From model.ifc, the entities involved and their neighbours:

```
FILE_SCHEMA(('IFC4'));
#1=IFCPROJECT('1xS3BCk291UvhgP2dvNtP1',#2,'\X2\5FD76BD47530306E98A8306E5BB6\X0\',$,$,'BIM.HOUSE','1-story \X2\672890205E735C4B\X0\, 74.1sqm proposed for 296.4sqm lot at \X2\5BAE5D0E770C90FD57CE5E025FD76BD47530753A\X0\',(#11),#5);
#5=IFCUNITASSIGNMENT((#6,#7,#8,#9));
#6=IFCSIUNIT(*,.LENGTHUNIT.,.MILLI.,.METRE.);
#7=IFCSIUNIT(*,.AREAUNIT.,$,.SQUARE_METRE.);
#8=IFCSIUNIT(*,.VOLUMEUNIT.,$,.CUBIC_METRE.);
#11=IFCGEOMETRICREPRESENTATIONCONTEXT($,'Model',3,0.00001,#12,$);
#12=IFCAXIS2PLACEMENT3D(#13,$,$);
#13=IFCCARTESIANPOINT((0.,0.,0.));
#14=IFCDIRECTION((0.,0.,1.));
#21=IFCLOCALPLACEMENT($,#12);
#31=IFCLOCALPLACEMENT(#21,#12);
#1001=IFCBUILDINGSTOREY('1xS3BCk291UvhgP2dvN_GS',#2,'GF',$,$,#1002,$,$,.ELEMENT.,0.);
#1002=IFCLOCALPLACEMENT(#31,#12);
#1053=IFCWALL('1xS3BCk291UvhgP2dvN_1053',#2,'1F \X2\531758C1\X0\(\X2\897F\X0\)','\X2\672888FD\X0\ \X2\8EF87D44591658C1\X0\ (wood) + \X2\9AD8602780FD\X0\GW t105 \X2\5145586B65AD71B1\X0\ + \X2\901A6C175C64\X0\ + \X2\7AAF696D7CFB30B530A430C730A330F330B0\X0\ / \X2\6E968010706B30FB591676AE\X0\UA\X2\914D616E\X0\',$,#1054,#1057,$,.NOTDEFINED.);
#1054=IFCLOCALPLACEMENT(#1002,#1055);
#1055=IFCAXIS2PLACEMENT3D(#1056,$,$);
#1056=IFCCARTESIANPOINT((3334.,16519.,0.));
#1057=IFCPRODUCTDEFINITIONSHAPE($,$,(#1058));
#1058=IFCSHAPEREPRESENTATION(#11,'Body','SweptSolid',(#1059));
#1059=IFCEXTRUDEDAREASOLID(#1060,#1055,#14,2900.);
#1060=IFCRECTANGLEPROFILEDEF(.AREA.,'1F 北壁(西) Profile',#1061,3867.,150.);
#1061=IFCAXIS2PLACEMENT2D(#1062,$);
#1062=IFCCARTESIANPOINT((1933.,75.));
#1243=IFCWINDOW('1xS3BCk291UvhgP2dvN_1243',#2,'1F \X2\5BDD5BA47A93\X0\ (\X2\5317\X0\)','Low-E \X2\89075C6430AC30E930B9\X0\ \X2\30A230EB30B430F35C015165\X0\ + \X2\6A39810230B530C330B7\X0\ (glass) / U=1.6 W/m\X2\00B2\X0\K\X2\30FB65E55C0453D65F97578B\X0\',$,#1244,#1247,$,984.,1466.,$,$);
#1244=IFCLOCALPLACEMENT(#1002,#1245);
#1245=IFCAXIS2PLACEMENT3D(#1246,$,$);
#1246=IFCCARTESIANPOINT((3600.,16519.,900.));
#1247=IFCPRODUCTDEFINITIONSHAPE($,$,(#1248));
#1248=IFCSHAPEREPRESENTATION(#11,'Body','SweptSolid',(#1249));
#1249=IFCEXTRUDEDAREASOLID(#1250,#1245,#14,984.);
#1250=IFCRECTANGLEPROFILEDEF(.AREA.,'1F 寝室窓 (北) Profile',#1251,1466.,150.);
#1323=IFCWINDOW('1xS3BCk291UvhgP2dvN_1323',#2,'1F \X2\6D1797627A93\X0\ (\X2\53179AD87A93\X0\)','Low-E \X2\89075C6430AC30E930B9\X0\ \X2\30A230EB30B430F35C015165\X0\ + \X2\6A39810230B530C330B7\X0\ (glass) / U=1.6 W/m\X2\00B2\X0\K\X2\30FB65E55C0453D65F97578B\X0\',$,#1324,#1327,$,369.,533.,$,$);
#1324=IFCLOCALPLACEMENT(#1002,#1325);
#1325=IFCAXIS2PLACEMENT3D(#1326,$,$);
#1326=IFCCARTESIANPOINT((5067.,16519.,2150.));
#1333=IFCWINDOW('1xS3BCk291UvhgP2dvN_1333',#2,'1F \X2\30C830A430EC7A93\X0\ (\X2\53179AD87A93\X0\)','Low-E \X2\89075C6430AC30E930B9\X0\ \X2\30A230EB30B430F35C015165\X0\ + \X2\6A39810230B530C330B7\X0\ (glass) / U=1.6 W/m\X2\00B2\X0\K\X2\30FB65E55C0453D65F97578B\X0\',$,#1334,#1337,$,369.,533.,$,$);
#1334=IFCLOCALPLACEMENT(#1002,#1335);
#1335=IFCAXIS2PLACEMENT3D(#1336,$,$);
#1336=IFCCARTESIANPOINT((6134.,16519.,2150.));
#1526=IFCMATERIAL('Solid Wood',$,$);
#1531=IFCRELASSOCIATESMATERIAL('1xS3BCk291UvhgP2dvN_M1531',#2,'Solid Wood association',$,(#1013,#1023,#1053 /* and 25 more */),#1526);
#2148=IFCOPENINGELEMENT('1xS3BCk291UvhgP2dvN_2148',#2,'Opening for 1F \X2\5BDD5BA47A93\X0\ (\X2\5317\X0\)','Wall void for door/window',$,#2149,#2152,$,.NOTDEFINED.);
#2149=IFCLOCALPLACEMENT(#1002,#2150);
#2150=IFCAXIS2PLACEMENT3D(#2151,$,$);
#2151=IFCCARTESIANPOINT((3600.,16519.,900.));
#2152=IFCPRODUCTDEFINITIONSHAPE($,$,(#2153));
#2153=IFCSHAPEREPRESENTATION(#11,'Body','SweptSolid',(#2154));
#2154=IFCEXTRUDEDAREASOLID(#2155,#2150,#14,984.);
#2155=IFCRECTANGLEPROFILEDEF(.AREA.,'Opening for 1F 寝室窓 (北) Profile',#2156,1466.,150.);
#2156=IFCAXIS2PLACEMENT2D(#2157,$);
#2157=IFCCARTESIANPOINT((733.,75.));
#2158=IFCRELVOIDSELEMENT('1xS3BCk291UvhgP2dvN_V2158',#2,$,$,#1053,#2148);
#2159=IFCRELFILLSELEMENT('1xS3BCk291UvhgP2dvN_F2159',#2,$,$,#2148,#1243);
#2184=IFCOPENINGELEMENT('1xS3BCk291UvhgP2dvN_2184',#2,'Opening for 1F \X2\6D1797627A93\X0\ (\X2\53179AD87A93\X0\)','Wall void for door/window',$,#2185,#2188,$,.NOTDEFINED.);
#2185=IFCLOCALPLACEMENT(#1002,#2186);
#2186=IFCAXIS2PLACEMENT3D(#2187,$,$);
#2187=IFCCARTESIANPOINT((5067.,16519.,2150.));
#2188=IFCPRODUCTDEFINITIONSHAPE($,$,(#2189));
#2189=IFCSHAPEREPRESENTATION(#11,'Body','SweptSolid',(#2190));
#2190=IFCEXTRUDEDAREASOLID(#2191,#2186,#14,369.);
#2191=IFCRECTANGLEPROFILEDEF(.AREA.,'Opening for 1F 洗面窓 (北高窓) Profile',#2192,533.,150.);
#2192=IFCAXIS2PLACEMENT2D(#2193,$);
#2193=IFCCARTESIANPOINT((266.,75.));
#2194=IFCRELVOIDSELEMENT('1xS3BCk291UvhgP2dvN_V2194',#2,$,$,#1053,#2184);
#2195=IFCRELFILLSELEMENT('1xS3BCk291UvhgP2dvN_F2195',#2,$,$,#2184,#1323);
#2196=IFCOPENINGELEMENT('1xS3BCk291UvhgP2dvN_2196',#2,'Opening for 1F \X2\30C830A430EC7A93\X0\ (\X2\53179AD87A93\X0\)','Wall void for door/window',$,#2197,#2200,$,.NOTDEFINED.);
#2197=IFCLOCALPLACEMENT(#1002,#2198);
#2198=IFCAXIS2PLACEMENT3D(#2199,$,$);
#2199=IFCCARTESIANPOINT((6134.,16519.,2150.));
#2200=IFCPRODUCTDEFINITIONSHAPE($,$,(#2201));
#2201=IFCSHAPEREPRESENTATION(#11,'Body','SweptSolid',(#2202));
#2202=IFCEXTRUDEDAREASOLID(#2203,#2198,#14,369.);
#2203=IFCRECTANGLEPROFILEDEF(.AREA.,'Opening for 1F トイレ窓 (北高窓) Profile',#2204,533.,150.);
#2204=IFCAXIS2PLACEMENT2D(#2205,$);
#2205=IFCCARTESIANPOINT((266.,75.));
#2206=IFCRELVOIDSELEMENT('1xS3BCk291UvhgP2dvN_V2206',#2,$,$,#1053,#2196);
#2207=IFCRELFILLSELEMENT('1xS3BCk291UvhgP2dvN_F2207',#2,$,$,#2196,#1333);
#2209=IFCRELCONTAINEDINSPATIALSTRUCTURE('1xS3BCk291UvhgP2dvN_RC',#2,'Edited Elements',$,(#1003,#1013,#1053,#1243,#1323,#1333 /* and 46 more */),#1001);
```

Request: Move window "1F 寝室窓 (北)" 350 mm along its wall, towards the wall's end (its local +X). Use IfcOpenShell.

```python
import ifcopenshell
import ifcopenshell.api.geometry
import ifcopenshell.util.placement
import ifcopenshell.util.unit

model = ifcopenshell.open("model.ifc")
unit_scale = ifcopenshell.util.unit.calculate_unit_scale(model)

window = model.by_id(1243)
opening = window.FillsVoids[0].RelatingOpeningElement
wall = opening.VoidsElements[0].RelatingBuildingElement

wall_matrix = ifcopenshell.util.placement.get_local_placement(wall.ObjectPlacement)
shift = wall_matrix[:3, 0] * 0.35 / unit_scale
before = ifcopenshell.util.placement.get_local_placement(window.ObjectPlacement)[:3, 3].copy()

# The window is not placed relative to its opening, so move both.
for product in (opening, window):
    matrix = ifcopenshell.util.placement.get_local_placement(product.ObjectPlacement)
    matrix[:3, 3] += shift
    ifcopenshell.api.geometry.edit_object_placement(model, product=product, matrix=matrix, is_si=False)

after = ifcopenshell.util.placement.get_local_placement(window.ObjectPlacement)[:3, 3]
print("window moved by", (after - before).round(3) + 0.0)

model.write("model_updated.ifc")
```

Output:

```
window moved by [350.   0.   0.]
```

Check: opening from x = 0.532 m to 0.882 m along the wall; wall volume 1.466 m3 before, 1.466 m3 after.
